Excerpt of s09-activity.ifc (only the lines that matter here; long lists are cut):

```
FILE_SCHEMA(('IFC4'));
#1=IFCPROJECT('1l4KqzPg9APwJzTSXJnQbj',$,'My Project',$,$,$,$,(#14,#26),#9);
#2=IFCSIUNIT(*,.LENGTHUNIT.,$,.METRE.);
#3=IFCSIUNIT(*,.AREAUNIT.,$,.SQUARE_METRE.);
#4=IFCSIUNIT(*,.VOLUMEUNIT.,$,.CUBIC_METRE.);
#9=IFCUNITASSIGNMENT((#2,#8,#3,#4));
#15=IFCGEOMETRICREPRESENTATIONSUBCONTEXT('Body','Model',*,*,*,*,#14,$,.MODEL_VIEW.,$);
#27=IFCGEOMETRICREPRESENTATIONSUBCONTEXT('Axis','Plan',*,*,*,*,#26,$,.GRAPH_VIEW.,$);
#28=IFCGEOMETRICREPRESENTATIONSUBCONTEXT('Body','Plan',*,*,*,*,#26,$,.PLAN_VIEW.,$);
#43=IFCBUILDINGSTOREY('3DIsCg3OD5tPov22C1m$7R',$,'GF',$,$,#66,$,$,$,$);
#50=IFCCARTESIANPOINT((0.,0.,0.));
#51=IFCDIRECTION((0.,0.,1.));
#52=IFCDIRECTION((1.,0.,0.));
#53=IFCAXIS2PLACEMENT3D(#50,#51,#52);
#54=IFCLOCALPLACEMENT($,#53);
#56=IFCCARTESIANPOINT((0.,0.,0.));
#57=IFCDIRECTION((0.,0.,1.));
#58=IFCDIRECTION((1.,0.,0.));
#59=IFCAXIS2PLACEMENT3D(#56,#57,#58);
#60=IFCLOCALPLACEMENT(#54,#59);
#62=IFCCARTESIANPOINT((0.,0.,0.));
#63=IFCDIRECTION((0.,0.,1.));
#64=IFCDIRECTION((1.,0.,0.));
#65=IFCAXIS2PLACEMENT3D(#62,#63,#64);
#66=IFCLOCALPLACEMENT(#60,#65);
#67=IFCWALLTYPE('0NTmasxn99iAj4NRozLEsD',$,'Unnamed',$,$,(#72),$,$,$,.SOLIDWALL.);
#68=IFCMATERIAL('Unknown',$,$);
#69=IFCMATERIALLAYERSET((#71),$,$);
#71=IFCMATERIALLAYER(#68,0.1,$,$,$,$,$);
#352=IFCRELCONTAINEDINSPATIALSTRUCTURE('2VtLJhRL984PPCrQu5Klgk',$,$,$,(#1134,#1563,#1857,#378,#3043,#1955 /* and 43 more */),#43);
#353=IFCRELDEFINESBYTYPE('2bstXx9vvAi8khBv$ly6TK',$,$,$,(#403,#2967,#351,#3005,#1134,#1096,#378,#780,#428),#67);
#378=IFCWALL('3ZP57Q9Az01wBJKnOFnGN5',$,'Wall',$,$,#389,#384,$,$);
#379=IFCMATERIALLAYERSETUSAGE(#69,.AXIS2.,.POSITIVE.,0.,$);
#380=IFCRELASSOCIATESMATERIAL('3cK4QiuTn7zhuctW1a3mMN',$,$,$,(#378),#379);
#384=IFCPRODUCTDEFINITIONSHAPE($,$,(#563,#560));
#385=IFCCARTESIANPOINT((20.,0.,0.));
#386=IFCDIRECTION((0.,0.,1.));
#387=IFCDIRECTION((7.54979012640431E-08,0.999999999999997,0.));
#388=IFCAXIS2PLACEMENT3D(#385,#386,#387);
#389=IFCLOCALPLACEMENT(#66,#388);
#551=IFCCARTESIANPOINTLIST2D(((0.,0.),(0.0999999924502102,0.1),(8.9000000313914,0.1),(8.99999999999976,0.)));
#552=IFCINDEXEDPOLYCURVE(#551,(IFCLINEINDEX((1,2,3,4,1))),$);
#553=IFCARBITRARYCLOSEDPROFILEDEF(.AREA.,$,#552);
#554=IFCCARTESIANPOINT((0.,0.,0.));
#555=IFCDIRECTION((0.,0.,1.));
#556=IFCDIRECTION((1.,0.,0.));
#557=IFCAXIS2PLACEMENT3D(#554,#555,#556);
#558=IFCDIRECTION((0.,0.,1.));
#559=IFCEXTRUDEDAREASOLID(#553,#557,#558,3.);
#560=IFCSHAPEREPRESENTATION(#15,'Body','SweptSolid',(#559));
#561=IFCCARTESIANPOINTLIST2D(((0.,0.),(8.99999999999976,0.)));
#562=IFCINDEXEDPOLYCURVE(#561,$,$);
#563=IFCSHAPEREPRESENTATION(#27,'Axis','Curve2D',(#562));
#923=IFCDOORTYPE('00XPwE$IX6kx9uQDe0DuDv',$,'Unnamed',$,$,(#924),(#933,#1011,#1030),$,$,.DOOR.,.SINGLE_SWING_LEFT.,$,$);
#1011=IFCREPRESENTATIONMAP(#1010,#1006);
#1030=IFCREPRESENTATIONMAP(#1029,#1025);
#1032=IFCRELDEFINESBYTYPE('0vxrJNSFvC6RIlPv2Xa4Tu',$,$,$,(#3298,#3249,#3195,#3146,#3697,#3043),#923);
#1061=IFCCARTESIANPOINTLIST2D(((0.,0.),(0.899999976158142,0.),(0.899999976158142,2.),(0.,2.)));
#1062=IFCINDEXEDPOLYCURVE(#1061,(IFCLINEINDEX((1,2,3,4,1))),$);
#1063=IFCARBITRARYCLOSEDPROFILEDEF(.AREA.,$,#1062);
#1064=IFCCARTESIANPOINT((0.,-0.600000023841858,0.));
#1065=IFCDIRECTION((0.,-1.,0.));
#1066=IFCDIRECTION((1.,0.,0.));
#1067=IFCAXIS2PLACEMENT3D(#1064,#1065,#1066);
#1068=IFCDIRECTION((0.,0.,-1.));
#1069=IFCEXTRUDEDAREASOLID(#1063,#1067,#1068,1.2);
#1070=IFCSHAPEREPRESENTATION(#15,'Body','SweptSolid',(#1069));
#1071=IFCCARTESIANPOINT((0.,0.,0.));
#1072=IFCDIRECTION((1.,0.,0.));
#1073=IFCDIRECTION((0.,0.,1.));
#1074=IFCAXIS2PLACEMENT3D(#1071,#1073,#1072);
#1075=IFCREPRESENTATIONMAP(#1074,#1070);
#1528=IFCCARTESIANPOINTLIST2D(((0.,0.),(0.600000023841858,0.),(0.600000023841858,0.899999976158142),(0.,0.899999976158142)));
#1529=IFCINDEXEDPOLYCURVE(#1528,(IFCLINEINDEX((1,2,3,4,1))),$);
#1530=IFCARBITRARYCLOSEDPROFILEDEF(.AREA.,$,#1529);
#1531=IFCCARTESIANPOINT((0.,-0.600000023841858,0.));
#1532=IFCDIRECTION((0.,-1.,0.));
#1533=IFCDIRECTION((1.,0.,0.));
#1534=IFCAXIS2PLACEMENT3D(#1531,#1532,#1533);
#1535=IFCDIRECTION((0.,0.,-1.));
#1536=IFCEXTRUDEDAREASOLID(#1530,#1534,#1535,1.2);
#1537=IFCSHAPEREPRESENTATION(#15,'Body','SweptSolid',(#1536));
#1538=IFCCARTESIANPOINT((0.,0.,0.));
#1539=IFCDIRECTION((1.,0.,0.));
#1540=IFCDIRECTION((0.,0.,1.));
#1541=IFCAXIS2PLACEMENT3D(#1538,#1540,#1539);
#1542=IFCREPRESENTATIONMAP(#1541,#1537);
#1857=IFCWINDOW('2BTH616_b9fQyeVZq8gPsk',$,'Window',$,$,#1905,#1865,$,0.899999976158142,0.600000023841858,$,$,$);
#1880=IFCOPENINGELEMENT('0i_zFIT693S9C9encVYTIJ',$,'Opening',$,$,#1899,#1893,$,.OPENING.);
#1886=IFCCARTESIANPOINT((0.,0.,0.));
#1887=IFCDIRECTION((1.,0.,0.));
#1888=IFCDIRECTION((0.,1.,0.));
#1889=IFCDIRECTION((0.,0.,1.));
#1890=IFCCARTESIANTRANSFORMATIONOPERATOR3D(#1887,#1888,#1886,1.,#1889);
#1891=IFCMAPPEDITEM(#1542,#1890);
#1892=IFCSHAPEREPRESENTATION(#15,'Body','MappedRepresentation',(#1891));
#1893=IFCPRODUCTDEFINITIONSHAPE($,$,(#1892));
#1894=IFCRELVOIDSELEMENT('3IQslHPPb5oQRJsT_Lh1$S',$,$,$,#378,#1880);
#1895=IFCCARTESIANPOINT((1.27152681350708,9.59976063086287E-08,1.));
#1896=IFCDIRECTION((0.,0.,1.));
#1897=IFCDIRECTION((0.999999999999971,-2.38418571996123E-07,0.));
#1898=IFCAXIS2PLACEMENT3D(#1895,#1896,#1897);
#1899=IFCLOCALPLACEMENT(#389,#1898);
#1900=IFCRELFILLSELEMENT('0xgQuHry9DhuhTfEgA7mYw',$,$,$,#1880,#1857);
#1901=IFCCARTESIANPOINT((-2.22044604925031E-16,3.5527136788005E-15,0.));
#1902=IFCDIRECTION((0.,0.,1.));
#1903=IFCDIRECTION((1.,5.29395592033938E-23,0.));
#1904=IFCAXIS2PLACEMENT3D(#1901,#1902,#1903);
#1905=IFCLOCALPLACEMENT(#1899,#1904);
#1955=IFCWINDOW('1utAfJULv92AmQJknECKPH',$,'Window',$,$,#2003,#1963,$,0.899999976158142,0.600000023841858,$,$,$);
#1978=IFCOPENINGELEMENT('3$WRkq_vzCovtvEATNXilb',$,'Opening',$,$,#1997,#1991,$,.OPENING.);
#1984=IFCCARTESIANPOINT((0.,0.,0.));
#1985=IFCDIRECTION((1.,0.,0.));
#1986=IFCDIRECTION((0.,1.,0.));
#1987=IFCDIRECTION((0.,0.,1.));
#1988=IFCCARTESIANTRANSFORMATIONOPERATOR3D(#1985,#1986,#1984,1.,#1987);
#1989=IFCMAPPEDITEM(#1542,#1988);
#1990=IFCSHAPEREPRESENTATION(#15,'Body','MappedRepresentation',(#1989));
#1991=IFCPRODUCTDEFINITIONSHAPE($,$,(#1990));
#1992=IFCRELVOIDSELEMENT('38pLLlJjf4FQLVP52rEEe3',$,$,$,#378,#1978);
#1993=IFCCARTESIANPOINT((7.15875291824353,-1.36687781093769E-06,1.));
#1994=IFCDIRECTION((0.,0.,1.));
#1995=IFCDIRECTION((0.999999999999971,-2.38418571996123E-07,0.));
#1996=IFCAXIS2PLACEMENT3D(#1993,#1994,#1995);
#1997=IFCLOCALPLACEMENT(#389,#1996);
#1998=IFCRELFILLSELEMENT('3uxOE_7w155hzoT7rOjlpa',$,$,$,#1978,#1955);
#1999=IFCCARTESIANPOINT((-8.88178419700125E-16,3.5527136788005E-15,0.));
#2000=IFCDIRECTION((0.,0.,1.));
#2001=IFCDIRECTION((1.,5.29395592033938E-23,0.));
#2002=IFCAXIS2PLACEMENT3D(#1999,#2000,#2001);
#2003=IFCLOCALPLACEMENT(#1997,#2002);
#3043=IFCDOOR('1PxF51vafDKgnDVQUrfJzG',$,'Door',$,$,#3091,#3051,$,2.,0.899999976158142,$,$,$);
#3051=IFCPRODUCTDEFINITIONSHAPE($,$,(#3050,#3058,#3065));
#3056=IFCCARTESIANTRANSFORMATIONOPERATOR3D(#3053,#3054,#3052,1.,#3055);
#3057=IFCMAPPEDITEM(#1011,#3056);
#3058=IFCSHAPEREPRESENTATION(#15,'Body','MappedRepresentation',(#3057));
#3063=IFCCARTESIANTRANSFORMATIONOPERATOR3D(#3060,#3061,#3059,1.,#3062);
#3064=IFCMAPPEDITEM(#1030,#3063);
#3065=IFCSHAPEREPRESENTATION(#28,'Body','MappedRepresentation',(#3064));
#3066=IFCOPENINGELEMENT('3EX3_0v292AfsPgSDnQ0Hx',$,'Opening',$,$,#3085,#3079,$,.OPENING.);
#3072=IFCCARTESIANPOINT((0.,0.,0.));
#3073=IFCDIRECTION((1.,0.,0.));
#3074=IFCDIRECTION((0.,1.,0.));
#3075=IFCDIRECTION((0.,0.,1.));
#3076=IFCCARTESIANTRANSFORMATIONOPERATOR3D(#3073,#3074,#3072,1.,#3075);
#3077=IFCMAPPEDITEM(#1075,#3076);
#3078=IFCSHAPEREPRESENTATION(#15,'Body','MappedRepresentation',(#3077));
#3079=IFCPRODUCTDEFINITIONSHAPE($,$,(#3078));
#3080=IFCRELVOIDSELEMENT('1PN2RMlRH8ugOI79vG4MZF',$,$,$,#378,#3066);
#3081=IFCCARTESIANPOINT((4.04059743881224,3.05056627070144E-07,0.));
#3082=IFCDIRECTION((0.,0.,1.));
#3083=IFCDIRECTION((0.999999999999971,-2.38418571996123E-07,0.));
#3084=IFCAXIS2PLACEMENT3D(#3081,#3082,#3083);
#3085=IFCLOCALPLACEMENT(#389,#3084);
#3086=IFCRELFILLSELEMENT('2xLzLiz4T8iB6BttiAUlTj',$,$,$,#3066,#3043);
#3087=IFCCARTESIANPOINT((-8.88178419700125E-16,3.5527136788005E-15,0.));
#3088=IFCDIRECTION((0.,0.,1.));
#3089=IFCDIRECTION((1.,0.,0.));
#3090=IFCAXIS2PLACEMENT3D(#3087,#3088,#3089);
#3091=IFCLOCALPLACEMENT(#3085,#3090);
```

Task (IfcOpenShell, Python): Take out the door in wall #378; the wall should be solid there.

```python
import ifcopenshell
import ifcopenshell.api.feature
import ifcopenshell.api.root
import ifcopenshell.geom
import ifcopenshell.util.shape

model = ifcopenshell.open("s09-activity.ifc")
settings = ifcopenshell.geom.settings()


def volume(element):
    """Net volume in cubic metres, openings subtracted."""
    shape = ifcopenshell.geom.create_shape(settings, element)
    return ifcopenshell.util.shape.get_volume(shape.geometry)


door = model.by_guid("1PxF51vafDKgnDVQUrfJzG")
opening = door.FillsVoids[0].RelatingOpeningElement
wall = opening.VoidsElements[0].RelatingBuildingElement
before = volume(wall)

ifcopenshell.api.root.remove_product(model, product=door)
ifcopenshell.api.feature.remove_feature(model, feature=opening)

after = volume(wall)

print(f"wall volume {before:.3f} -> {after:.3f} m3")

model.write("s09-activity_v2.ifc")
```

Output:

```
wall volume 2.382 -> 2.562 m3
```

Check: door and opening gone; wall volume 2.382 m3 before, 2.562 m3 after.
